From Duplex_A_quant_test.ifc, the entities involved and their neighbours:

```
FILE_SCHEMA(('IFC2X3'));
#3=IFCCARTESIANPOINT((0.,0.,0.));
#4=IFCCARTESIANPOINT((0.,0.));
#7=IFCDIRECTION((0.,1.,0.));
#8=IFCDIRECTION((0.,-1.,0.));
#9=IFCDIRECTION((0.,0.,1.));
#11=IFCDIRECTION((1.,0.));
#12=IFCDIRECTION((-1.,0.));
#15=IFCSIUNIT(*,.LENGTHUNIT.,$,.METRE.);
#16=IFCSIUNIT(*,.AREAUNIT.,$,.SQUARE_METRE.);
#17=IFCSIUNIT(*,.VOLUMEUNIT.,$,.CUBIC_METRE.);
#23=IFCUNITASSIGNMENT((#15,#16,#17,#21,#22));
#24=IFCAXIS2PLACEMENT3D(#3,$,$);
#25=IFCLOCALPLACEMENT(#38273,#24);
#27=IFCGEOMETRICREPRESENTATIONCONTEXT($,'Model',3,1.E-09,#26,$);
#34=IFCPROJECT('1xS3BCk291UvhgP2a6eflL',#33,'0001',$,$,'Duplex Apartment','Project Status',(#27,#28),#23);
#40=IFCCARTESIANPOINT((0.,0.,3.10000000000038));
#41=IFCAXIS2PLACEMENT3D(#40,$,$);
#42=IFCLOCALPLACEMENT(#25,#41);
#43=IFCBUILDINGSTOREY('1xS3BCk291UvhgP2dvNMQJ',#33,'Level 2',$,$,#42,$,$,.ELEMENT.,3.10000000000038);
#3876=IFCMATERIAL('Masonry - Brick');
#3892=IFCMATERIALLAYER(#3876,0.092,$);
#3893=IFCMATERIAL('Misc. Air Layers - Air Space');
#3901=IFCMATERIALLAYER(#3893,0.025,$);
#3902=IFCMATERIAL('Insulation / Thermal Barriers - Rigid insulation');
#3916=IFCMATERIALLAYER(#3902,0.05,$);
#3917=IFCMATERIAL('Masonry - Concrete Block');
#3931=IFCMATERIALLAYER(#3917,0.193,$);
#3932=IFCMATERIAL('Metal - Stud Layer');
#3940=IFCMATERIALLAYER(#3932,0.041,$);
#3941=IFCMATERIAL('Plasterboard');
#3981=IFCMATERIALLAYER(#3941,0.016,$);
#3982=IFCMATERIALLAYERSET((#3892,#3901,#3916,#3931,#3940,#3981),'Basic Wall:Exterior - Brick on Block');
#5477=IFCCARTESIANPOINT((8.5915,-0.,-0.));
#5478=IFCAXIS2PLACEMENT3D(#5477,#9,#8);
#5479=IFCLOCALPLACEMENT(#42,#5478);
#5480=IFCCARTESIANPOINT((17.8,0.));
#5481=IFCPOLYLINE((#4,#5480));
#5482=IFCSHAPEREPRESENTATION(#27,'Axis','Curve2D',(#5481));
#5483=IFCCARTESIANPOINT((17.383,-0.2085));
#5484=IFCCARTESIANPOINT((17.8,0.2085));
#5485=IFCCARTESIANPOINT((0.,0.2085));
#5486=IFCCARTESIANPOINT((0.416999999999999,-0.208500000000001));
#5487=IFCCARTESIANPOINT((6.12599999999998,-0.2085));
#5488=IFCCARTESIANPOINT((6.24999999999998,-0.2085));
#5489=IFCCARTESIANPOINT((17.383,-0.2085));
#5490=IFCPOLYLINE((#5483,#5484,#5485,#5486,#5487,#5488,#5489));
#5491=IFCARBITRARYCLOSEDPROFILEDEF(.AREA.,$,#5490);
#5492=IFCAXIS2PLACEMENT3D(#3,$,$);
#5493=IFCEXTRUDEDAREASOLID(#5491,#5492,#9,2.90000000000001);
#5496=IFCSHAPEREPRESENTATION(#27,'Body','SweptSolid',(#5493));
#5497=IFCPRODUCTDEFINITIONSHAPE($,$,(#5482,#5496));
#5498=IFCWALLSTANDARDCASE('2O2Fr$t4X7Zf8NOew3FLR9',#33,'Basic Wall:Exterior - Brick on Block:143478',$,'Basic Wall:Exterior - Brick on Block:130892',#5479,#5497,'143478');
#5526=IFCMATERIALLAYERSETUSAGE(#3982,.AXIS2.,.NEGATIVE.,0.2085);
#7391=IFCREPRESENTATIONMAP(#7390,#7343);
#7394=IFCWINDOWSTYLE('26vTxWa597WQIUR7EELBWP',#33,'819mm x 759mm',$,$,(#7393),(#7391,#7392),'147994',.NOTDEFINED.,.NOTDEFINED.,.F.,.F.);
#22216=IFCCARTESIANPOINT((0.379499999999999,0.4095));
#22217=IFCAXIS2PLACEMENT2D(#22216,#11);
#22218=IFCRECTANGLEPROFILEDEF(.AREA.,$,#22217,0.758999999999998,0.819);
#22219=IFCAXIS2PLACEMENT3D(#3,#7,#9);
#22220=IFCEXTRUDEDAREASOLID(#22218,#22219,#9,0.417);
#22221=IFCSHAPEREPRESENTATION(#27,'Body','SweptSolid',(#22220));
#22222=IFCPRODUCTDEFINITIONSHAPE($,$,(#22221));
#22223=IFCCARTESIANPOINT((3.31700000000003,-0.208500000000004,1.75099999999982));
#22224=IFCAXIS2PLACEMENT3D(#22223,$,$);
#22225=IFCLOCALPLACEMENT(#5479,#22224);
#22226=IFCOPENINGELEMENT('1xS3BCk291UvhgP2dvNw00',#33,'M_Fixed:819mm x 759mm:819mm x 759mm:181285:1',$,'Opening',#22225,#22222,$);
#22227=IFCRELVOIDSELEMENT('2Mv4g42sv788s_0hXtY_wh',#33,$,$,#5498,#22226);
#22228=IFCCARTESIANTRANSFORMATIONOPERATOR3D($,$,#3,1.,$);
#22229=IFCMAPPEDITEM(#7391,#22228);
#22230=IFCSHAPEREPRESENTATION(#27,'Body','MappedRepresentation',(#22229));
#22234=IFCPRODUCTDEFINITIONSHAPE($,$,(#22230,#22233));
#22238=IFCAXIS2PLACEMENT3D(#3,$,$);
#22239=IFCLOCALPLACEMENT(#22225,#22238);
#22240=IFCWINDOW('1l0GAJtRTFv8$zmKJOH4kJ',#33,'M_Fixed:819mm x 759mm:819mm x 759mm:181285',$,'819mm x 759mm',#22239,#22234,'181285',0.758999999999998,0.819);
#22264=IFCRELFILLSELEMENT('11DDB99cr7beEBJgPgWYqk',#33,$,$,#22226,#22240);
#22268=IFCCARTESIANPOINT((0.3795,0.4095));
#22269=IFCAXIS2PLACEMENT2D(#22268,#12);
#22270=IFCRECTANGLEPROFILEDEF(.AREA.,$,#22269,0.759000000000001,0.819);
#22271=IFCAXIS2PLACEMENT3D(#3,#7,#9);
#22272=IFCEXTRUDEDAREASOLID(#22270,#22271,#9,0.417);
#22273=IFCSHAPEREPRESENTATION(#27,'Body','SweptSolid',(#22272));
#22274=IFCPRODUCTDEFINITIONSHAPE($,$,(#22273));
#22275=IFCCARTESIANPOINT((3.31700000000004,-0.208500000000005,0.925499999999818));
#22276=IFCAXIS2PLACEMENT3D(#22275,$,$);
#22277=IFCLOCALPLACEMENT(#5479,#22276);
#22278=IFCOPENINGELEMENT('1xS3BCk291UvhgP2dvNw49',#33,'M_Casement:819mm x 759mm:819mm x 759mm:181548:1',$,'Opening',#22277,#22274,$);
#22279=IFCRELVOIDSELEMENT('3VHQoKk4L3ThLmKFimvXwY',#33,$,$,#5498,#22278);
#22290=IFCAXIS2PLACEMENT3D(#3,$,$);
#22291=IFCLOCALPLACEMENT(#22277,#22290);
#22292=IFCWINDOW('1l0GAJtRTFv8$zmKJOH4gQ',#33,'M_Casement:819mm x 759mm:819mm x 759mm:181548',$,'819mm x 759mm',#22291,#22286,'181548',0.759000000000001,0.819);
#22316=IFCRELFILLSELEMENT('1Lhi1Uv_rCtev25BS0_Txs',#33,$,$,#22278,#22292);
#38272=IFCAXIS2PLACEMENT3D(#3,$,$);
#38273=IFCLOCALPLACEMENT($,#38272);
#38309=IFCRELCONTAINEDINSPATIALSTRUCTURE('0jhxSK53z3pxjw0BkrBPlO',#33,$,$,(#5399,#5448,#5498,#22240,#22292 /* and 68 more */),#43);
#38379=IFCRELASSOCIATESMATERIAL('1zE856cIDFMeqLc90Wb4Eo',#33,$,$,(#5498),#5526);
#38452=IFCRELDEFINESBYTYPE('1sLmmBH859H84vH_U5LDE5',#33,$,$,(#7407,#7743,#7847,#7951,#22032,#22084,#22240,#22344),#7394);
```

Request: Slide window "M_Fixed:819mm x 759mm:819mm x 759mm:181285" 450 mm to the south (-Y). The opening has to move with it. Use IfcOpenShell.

```python
import ifcopenshell
import ifcopenshell.api.geometry
import ifcopenshell.util.placement
import ifcopenshell.util.unit

model = ifcopenshell.open("Duplex_A_quant_test.ifc")
unit_scale = ifcopenshell.util.unit.calculate_unit_scale(model)

window = model.by_guid("1l0GAJtRTFv8$zmKJOH4kJ")
opening = window.FillsVoids[0].RelatingOpeningElement
wall = opening.VoidsElements[0].RelatingBuildingElement

wall_matrix = ifcopenshell.util.placement.get_local_placement(wall.ObjectPlacement)
shift = wall_matrix[:3, 0] * 0.45 / unit_scale
before = ifcopenshell.util.placement.get_local_placement(window.ObjectPlacement)[:3, 3].copy()

# The window is placed relative to its opening, so it follows when the opening moves.
matrix = ifcopenshell.util.placement.get_local_placement(opening.ObjectPlacement)
matrix[:3, 3] += shift
ifcopenshell.api.geometry.edit_object_placement(
    model, product=opening, matrix=matrix, is_si=False, should_transform_children=True
)

after = ifcopenshell.util.placement.get_local_placement(window.ObjectPlacement)[:3, 3]
print("window moved by", (after - before).round(3) + 0.0)

model.write("Duplex_A_quant_test_rev.ifc")
```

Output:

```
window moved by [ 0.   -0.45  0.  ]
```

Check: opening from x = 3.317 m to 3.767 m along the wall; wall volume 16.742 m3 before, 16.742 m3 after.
